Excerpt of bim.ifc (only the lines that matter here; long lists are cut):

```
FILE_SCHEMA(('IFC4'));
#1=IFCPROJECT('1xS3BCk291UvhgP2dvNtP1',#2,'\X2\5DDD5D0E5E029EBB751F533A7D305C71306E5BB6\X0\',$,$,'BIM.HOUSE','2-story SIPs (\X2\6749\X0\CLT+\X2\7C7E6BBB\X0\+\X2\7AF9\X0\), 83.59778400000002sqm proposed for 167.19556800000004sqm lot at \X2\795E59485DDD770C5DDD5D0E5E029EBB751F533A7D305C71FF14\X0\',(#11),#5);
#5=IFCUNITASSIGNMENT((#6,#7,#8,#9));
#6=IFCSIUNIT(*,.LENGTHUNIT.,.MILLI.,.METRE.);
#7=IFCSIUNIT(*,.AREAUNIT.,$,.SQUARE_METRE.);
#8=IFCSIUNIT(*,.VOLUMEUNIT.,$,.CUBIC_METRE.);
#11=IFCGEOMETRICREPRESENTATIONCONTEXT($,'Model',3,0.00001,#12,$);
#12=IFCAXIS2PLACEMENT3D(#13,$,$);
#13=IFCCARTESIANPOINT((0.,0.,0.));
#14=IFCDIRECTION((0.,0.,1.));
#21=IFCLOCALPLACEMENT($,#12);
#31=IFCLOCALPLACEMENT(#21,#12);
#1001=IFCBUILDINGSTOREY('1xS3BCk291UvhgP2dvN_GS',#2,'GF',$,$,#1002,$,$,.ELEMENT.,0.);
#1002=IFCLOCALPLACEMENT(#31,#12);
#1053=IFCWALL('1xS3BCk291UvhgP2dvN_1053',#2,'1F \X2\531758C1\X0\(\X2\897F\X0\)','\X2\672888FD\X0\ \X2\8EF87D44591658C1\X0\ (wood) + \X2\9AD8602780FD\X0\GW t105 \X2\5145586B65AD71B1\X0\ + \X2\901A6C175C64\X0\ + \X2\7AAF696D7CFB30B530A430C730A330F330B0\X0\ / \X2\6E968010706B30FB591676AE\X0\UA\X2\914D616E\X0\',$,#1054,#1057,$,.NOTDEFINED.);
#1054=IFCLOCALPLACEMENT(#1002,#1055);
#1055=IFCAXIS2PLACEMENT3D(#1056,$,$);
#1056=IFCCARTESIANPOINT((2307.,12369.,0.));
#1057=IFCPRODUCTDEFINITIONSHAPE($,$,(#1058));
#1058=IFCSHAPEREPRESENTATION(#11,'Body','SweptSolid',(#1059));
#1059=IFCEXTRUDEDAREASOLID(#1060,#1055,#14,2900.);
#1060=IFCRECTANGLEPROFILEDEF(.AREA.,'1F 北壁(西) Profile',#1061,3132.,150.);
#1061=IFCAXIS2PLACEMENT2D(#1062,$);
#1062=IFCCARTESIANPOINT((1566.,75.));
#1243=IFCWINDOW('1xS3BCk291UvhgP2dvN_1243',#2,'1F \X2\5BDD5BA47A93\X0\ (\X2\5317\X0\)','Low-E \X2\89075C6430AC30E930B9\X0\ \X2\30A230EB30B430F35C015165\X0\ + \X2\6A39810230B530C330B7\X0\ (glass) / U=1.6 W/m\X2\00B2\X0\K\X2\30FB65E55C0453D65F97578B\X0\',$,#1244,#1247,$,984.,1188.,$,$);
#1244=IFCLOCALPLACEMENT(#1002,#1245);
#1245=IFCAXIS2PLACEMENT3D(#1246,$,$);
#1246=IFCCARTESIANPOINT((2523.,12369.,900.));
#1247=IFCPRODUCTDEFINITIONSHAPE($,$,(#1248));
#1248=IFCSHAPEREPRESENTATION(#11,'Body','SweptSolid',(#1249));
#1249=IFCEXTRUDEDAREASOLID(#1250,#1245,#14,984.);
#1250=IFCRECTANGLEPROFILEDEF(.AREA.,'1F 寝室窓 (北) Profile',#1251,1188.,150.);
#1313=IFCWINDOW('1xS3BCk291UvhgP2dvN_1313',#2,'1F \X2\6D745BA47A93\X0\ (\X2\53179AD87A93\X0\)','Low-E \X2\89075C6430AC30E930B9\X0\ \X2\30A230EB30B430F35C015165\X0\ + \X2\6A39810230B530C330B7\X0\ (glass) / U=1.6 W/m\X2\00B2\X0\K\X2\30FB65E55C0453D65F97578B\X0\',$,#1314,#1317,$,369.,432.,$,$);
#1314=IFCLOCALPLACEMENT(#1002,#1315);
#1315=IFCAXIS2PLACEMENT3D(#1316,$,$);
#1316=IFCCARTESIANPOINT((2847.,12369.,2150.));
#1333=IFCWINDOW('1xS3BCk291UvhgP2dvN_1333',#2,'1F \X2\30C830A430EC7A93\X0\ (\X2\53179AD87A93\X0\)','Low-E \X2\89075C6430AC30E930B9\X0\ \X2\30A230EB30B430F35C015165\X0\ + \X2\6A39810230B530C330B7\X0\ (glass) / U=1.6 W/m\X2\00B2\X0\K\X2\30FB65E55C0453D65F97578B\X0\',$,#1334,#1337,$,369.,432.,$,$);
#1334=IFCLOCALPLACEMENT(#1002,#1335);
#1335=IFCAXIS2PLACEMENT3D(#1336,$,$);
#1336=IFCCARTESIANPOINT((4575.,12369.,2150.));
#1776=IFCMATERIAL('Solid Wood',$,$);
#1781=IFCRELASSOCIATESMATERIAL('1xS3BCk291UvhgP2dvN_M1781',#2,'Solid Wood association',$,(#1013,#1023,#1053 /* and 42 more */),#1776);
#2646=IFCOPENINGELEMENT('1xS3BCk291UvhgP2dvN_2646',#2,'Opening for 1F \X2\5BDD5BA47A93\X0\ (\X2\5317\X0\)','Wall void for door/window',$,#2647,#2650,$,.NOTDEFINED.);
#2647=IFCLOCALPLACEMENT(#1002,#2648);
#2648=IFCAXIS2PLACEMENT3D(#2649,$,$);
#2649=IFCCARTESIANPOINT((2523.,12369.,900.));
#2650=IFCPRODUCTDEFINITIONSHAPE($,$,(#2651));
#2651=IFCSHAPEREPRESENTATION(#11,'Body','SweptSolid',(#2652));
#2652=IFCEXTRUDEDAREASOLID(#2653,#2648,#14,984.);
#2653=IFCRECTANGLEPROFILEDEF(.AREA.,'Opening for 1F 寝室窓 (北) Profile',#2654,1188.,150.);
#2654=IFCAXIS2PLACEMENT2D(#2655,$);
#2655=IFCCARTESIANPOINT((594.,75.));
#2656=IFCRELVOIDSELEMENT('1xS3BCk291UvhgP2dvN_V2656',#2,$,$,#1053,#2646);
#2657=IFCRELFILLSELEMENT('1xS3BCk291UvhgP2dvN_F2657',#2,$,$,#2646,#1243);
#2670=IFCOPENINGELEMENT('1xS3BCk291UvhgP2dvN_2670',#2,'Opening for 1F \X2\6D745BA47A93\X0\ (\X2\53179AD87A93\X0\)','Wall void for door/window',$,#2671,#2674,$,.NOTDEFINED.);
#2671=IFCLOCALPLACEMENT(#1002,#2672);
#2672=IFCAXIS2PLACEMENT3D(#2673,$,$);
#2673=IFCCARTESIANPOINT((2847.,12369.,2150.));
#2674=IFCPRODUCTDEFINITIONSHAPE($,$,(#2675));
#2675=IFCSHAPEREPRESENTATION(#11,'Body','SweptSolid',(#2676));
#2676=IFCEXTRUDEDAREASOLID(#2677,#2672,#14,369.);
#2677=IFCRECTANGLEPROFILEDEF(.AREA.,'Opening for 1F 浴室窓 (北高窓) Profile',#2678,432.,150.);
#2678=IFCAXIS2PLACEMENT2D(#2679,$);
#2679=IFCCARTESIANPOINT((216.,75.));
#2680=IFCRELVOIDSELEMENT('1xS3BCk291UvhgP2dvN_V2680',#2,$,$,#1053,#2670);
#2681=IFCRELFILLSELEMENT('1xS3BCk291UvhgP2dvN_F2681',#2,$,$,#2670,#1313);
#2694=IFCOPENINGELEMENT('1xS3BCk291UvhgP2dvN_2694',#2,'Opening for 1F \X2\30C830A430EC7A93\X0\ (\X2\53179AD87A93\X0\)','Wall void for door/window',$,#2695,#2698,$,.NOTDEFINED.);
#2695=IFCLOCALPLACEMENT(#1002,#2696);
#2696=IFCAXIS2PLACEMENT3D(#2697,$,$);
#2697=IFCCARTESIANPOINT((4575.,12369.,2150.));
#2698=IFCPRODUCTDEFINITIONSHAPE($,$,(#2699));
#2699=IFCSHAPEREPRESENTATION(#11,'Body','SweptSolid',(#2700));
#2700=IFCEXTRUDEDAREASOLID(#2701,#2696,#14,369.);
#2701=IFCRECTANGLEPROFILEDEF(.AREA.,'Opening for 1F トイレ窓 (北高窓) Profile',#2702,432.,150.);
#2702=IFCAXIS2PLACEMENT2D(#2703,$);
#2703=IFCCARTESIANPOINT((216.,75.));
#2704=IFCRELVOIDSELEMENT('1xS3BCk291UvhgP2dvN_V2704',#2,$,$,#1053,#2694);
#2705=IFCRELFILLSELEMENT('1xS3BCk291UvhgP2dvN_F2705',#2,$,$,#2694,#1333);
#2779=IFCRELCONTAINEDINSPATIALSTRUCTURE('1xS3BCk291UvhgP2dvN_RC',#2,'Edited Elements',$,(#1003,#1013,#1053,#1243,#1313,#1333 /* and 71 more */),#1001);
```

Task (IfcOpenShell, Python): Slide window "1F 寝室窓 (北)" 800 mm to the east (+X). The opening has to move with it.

```python
import ifcopenshell
import ifcopenshell.api.geometry
import ifcopenshell.util.placement
import ifcopenshell.util.unit

model = ifcopenshell.open("bim.ifc")
unit_scale = ifcopenshell.util.unit.calculate_unit_scale(model)

window = model.by_id(1243)
opening = window.FillsVoids[0].RelatingOpeningElement
wall = opening.VoidsElements[0].RelatingBuildingElement

wall_matrix = ifcopenshell.util.placement.get_local_placement(wall.ObjectPlacement)
shift = wall_matrix[:3, 0] * 0.8 / unit_scale
before = ifcopenshell.util.placement.get_local_placement(window.ObjectPlacement)[:3, 3].copy()

# The window is not placed relative to its opening, so move both.
for product in (opening, window):
    matrix = ifcopenshell.util.placement.get_local_placement(product.ObjectPlacement)
    matrix[:3, 3] += shift
    ifcopenshell.api.geometry.edit_object_placement(model, product=product, matrix=matrix, is_si=False)

after = ifcopenshell.util.placement.get_local_placement(window.ObjectPlacement)[:3, 3]
print("window moved by", (after - before).round(3) + 0.0)

model.write("bim-out.ifc")
```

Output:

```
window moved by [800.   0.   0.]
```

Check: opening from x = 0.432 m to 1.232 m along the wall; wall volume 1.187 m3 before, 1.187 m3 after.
